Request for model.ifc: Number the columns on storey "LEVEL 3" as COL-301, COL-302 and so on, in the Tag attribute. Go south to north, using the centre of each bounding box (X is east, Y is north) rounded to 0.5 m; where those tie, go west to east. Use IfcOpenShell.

First a look at what the model holds.

```python
import ifcopenshell
import ifcopenshell.util.element
import ifcopenshell.util.placement

model = ifcopenshell.open("model.ifc")
print(model.schema)
storey = next(s for s in model.by_type("IfcBuildingStorey") if s.Name == "LEVEL 3")
columns = [e for e in ifcopenshell.util.element.get_decomposition(storey) if e.is_a("IfcColumn")]
for e in sorted(columns, key=lambda e: e.id()):
    origin = ifcopenshell.util.placement.get_local_placement(e.ObjectPlacement)[:3, 3]
    print(e.id(), e.Tag, e.Name, origin.round(2) + 0.0, sep=" | ")
```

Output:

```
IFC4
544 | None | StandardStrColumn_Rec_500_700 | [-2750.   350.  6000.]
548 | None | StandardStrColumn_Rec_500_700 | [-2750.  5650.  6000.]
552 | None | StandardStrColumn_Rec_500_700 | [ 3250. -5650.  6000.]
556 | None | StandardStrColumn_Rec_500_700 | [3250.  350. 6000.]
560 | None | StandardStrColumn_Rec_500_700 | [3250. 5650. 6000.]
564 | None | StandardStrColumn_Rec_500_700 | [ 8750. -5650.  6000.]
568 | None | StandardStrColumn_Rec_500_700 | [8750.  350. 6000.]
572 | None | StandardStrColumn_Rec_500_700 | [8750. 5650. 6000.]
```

```python
import ifcopenshell
import ifcopenshell.geom
import ifcopenshell.util.element
import ifcopenshell.util.shape

model = ifcopenshell.open("model.ifc")
settings = ifcopenshell.geom.settings()
settings.set("use-world-coords", True)


def centre(element):
    shape = ifcopenshell.geom.create_shape(settings, element)
    return ifcopenshell.util.shape.get_bbox_centroid(shape.geometry)


storey = next(s for s in model.by_type("IfcBuildingStorey") if s.Name == "LEVEL 3")
columns = [e for e in ifcopenshell.util.element.get_decomposition(storey) if e.is_a("IfcColumn")]

# Insertion points can sit at a corner or the storey origin, so sort by the geometry (in metres).
centres = {e: centre(e) for e in columns}
columns.sort(key=lambda e: (round(centres[e][1] / 0.5), centres[e][0]))

for i, e in enumerate(columns, start=1):
    number = f"COL-3{i:02d}"
    e.Tag = number
    print(e.id(), number)

model.write("model_v2.ifc")
```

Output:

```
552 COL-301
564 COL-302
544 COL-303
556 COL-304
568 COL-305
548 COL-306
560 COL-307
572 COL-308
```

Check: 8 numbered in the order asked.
